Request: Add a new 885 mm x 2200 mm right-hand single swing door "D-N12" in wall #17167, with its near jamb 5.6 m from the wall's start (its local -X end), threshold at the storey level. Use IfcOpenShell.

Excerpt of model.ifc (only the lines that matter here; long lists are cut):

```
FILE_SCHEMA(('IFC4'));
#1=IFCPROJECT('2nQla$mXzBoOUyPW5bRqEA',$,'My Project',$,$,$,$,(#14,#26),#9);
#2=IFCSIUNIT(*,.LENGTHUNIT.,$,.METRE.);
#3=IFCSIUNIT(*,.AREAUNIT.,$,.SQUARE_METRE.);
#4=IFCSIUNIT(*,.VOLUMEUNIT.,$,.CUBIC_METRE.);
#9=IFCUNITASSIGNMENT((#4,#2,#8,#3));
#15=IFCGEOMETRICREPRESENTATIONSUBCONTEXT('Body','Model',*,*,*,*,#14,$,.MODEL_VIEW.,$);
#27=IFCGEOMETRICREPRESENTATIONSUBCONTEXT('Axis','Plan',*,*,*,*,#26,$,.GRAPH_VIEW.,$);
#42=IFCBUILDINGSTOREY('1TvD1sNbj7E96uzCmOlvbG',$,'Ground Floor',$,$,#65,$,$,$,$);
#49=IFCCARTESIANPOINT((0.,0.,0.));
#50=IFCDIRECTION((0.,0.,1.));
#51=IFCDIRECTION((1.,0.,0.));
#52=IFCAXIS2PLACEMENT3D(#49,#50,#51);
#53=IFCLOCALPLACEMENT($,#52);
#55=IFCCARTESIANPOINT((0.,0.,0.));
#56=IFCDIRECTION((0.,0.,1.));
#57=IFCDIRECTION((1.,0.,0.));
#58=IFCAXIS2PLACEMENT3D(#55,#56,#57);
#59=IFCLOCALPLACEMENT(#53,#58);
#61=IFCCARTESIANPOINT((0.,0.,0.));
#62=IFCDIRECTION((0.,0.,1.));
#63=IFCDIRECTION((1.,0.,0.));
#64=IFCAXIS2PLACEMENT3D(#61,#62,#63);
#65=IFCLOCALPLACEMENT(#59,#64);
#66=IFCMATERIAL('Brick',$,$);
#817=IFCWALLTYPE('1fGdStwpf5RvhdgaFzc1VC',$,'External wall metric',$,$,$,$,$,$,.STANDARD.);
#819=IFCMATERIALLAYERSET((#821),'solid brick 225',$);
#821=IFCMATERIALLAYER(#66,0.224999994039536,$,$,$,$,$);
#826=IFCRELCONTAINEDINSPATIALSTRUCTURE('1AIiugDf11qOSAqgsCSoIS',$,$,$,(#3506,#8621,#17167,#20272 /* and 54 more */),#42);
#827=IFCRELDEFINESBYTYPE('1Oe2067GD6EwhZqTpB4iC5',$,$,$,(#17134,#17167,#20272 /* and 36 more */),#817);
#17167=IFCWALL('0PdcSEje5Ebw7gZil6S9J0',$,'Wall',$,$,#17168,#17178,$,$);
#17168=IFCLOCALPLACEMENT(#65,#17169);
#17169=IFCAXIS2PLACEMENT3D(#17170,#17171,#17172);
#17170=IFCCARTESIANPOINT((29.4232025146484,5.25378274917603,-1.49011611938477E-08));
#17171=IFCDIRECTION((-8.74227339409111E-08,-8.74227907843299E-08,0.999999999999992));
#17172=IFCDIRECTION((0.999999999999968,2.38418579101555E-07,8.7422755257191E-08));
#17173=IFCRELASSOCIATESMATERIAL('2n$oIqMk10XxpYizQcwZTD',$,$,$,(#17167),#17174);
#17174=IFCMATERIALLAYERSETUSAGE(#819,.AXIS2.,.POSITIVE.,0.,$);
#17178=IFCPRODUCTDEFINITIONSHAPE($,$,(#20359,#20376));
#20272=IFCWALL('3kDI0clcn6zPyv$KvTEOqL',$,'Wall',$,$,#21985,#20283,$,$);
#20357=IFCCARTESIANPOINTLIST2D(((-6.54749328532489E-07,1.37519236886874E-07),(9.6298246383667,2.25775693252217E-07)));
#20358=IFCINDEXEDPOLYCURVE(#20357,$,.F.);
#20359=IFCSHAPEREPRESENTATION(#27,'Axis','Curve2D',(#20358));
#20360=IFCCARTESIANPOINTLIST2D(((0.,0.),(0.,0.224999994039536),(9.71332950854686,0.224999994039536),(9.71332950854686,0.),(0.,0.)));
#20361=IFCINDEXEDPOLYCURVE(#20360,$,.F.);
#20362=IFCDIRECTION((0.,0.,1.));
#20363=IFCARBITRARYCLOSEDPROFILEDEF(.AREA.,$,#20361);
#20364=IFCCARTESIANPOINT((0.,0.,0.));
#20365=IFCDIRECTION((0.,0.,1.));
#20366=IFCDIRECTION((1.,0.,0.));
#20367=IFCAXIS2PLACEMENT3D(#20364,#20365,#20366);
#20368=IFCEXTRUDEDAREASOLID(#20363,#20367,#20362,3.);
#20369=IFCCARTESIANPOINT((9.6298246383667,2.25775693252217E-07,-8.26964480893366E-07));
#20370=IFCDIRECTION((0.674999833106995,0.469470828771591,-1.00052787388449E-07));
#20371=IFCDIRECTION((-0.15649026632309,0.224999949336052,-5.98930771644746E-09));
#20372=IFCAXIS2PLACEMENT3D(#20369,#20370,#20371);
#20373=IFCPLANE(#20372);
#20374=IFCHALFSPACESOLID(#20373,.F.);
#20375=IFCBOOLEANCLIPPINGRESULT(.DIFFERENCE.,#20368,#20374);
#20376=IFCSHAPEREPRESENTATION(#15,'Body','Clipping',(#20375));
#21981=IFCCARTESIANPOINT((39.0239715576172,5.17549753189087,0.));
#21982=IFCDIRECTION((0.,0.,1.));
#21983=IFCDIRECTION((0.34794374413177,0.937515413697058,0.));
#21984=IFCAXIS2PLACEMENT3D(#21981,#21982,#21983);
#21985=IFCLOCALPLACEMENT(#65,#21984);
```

```python
import numpy as np
import ifcopenshell
import ifcopenshell.api.feature
import ifcopenshell.api.geometry
import ifcopenshell.api.root
import ifcopenshell.api.spatial
import ifcopenshell.geom
import ifcopenshell.util.element
import ifcopenshell.util.placement
import ifcopenshell.util.representation
import ifcopenshell.util.shape
import ifcopenshell.util.unit

model = ifcopenshell.open("model.ifc")
unit_scale = ifcopenshell.util.unit.calculate_unit_scale(model)
settings = ifcopenshell.geom.settings()


def volume(element):
    """Net volume in cubic metres, openings subtracted."""
    shape = ifcopenshell.geom.create_shape(settings, element)
    return ifcopenshell.util.shape.get_volume(shape.geometry)


wall = model.by_id(17167)
storey = ifcopenshell.util.element.get_container(wall, ifc_class="IfcBuildingStorey")
context = ifcopenshell.util.representation.get_context(model, "Model", "Body", "MODEL_VIEW")
before = volume(wall)

width, height, from_end, sill = 0.885, 2.2, 5.6, 0.0  # metres

# The wall runs along its own X axis, and the end named is its -X end.
wall_shape = ifcopenshell.geom.create_shape(settings, wall)
x, y, z = ifcopenshell.util.shape.get_vertices(wall_shape.geometry).T
start = x.min() + from_end
face, thickness = float(y.min()), float(y.max() - y.min())
wall_matrix = ifcopenshell.util.placement.get_local_placement(wall.ObjectPlacement)
level = ifcopenshell.util.placement.get_local_placement(storey.ObjectPlacement)[2, 3]


def in_wall(x, y):
    """Placement at x, y metres in the wall's axes, at sill height."""
    matrix = wall_matrix.copy()
    matrix[:, 3] = wall_matrix @ np.array([x / unit_scale, y / unit_scale, 0.0, 1.0])
    matrix[2, 3] = level + sill / unit_scale
    return matrix


# Opening: a box that overshoots both wall faces by 50 mm.
opening = ifcopenshell.api.root.create_entity(model, ifc_class="IfcOpeningElement", predefined_type="OPENING")
box = ifcopenshell.api.geometry.add_wall_representation(
    model, context=context, length=width, height=height, thickness=thickness + 0.1
)
ifcopenshell.api.geometry.assign_representation(model, product=opening, representation=box)
ifcopenshell.api.geometry.edit_object_placement(model, product=opening, matrix=in_wall(start, face - 0.05), is_si=False)
ifcopenshell.api.feature.add_feature(model, feature=opening, element=wall)

door = ifcopenshell.api.root.create_entity(model, ifc_class="IfcDoor", name="D-N12", predefined_type="DOOR")
door.OverallWidth, door.OverallHeight = width / unit_scale, height / unit_scale
door.OperationType = "SINGLE_SWING_RIGHT"
body = ifcopenshell.api.geometry.add_door_representation(
    model,
    context=context,
    overall_width=door.OverallWidth,
    overall_height=door.OverallHeight,
    operation_type="SINGLE_SWING_RIGHT",
    lining_properties={"LiningDepth": thickness / unit_scale, "ThresholdDepth": thickness / unit_scale},
)
ifcopenshell.api.geometry.assign_representation(model, product=door, representation=body)
ifcopenshell.api.spatial.assign_container(model, products=[door], relating_structure=storey)
ifcopenshell.api.feature.add_filling(model, opening=opening, element=door)

# The lining spans the wall, so the door starts at the wall face.
ifcopenshell.api.geometry.edit_object_placement(model, product=door, matrix=in_wall(start, face), is_si=False)

after = volume(wall)

print(f"wall volume {before:.3f} -> {after:.3f} m3")

model.write("model_v2.ifc")
```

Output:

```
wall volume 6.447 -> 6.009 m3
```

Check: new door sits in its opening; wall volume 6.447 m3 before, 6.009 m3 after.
